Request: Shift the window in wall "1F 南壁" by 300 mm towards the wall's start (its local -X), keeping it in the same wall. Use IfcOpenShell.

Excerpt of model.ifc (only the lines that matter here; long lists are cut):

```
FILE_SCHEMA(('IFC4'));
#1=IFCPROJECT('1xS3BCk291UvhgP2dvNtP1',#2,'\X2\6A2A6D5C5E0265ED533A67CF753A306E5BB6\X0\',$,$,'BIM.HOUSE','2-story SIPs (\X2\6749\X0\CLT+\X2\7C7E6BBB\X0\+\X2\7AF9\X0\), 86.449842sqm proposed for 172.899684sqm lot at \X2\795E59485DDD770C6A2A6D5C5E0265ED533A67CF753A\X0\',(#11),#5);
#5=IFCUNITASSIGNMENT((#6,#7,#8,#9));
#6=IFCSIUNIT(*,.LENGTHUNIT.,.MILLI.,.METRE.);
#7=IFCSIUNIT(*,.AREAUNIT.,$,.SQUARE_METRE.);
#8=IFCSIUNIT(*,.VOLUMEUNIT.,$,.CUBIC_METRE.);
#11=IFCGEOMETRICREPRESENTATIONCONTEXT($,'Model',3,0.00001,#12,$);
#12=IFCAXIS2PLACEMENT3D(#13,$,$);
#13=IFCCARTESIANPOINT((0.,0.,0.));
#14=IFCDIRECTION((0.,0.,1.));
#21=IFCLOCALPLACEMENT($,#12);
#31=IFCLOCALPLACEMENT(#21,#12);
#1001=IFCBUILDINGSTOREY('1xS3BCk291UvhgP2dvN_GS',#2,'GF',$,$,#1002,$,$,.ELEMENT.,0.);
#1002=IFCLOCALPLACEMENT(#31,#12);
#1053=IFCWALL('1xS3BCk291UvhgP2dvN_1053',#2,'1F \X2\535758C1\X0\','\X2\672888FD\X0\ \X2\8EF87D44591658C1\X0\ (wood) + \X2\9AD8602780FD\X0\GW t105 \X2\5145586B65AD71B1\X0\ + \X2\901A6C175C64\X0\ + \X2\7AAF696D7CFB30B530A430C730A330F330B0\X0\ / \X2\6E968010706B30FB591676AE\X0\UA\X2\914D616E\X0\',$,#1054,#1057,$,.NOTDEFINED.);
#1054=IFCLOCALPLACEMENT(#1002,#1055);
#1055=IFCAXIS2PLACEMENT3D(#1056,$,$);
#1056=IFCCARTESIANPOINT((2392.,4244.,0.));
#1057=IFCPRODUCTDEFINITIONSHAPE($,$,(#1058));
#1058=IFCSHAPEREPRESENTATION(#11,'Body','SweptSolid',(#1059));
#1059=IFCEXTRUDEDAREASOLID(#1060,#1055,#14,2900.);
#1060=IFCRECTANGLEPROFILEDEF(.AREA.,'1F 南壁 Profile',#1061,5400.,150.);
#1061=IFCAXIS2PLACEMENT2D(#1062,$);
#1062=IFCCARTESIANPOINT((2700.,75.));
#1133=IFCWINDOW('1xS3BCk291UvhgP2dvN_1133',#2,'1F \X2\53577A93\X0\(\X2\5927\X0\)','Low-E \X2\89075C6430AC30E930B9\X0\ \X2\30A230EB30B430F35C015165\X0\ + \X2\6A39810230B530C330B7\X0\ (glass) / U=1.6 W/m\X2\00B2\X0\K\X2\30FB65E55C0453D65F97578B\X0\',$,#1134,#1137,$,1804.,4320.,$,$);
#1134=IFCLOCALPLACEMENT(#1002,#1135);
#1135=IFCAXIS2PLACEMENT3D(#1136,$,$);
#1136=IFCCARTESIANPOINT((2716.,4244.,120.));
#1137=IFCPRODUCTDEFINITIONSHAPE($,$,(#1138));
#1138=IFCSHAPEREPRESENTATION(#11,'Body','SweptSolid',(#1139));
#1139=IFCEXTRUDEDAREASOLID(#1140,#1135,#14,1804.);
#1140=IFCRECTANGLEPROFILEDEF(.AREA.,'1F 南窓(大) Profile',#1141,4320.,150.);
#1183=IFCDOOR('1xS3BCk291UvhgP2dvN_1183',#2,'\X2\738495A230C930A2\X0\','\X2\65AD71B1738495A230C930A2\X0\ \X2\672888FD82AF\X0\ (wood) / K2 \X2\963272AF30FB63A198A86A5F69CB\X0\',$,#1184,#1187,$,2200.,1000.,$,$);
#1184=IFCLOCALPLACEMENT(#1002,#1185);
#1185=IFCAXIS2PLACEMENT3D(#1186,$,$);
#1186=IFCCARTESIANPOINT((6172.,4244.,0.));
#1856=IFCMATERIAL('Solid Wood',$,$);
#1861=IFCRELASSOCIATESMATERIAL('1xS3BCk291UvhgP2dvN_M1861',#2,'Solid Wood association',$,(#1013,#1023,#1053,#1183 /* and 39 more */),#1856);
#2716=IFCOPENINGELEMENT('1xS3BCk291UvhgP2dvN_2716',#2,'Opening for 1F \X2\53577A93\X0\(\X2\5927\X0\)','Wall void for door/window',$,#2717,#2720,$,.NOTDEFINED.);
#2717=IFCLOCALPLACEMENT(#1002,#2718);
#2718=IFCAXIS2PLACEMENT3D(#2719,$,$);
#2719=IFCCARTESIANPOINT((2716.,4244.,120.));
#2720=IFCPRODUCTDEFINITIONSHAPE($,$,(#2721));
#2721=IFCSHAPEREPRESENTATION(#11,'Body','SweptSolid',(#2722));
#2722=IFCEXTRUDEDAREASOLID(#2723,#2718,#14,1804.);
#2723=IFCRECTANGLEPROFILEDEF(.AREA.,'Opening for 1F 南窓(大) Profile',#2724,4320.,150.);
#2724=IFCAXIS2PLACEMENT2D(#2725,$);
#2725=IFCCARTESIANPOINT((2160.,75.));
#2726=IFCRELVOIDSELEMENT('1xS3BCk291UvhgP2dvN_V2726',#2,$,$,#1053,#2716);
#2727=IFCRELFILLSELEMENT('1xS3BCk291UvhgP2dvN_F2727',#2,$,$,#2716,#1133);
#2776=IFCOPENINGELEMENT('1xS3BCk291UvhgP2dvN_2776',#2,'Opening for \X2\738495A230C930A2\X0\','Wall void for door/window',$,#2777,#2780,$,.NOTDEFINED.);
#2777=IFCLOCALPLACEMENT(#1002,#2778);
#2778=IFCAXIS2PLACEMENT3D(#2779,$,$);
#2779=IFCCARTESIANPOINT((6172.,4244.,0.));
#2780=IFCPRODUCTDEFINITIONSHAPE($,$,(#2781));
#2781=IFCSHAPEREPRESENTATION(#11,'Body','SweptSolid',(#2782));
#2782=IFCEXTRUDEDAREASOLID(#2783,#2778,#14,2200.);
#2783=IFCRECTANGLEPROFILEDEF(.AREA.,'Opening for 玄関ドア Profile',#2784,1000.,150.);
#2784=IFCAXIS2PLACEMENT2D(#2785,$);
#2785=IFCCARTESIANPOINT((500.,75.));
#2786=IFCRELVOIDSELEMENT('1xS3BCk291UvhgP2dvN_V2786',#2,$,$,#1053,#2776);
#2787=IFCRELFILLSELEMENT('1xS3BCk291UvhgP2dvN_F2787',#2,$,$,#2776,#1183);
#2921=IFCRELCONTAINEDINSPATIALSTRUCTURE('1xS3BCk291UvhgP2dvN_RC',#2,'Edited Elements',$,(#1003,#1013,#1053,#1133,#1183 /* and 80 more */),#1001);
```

```python
import ifcopenshell
import ifcopenshell.api.geometry
import ifcopenshell.util.placement

model = ifcopenshell.open("model.ifc")

window = model.by_guid("1xS3BCk291UvhgP2dvN_1133")
opening = window.FillsVoids[0].RelatingOpeningElement
wall = opening.VoidsElements[0].RelatingBuildingElement

wall_matrix = ifcopenshell.util.placement.get_local_placement(wall.ObjectPlacement)
shift = wall_matrix[:3, 0] * -300.0
before = ifcopenshell.util.placement.get_local_placement(window.ObjectPlacement)[:3, 3].copy()

# The window is not placed relative to its opening, so move both.
for product in (opening, window):
    matrix = ifcopenshell.util.placement.get_local_placement(product.ObjectPlacement)
    matrix[:3, 3] += shift
    ifcopenshell.api.geometry.edit_object_placement(model, product=product, matrix=matrix, is_si=False)

after = ifcopenshell.util.placement.get_local_placement(window.ObjectPlacement)[:3, 3]
print("window moved by", (after - before).round(3) + 0.0)

model.write("model_rev.ifc")
```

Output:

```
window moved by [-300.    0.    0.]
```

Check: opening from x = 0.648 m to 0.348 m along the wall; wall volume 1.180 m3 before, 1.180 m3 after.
